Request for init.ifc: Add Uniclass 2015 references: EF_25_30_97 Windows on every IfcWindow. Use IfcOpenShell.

First a look at what the model holds.

```python
import ifcopenshell

model = ifcopenshell.open("init.ifc")
print(model.schema)
print("classifications:", [c.Name for c in model.by_type("IfcClassification")])
for ifc_class in ("IfcDoor", "IfcRoof", "IfcStair", "IfcWall", "IfcWindow"):
    print(ifc_class, len(model.by_type(ifc_class)))
```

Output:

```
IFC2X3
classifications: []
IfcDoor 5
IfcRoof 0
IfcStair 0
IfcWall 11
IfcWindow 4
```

```python
import ifcopenshell
import ifcopenshell.api.classification

model = ifcopenshell.open("init.ifc")

# IFC2X3 requires Source and Edition and has no link from the project to the system.
system = model.create_entity("IfcClassification", Source="NBS", Edition="2015", Name="Uniclass 2015")

codes = {
    "IfcWindow": ("EF_25_30_97", "Windows"),
}
for ifc_class, (code, name) in codes.items():
    products = model.by_type(ifc_class)
    ifcopenshell.api.classification.add_reference(
        model, products=products, classification=system, identification=code, name=name
    )
    print(code, len(products))

model.write("init_rev.ifc")
```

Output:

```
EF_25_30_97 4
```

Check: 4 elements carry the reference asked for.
